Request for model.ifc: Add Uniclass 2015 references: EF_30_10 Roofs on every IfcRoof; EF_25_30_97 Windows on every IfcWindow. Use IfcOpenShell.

First a look at what the model holds.

```python
import ifcopenshell

model = ifcopenshell.open("model.ifc")
print(model.schema)
print("classifications:", [c.Name for c in model.by_type("IfcClassification")])
for ifc_class in ("IfcDoor", "IfcRoof", "IfcStair", "IfcWall", "IfcWindow"):
    print(ifc_class, len(model.by_type(ifc_class)))
```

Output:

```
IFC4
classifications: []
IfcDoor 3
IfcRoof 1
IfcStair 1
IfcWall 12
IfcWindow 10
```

```python
import ifcopenshell
import ifcopenshell.api.classification

model = ifcopenshell.open("model.ifc")

system = ifcopenshell.api.classification.add_classification(model, classification="Uniclass 2015")

codes = {
    "IfcRoof": ("EF_30_10", "Roofs"),
    "IfcWindow": ("EF_25_30_97", "Windows"),
}
for ifc_class, (code, name) in codes.items():
    products = model.by_type(ifc_class)
    ifcopenshell.api.classification.add_reference(
        model, products=products, classification=system, identification=code, name=name
    )
    print(code, len(products))

model.write("model_updated.ifc")
```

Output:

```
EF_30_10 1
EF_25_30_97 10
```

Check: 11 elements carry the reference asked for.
